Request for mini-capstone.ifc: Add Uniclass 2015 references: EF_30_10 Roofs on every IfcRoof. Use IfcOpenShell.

First a look at what the model holds.

```python
import ifcopenshell

model = ifcopenshell.open("mini-capstone.ifc")
print(model.schema)
print("classifications:", [c.Name for c in model.by_type("IfcClassification")])
for ifc_class in ("IfcDoor", "IfcRoof", "IfcStair", "IfcWall", "IfcWindow"):
    print(ifc_class, len(model.by_type(ifc_class)))
```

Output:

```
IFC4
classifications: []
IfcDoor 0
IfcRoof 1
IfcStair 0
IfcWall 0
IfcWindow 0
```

```python
import ifcopenshell
import ifcopenshell.api.classification

model = ifcopenshell.open("mini-capstone.ifc")

system = ifcopenshell.api.classification.add_classification(model, classification="Uniclass 2015")

codes = {
    "IfcRoof": ("EF_30_10", "Roofs"),
}
for ifc_class, (code, name) in codes.items():
    products = model.by_type(ifc_class)
    ifcopenshell.api.classification.add_reference(
        model, products=products, classification=system, identification=code, name=name
    )
    print(code, len(products))

model.write("mini-capstone_v2.ifc")
```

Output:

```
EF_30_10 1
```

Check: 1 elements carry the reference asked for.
